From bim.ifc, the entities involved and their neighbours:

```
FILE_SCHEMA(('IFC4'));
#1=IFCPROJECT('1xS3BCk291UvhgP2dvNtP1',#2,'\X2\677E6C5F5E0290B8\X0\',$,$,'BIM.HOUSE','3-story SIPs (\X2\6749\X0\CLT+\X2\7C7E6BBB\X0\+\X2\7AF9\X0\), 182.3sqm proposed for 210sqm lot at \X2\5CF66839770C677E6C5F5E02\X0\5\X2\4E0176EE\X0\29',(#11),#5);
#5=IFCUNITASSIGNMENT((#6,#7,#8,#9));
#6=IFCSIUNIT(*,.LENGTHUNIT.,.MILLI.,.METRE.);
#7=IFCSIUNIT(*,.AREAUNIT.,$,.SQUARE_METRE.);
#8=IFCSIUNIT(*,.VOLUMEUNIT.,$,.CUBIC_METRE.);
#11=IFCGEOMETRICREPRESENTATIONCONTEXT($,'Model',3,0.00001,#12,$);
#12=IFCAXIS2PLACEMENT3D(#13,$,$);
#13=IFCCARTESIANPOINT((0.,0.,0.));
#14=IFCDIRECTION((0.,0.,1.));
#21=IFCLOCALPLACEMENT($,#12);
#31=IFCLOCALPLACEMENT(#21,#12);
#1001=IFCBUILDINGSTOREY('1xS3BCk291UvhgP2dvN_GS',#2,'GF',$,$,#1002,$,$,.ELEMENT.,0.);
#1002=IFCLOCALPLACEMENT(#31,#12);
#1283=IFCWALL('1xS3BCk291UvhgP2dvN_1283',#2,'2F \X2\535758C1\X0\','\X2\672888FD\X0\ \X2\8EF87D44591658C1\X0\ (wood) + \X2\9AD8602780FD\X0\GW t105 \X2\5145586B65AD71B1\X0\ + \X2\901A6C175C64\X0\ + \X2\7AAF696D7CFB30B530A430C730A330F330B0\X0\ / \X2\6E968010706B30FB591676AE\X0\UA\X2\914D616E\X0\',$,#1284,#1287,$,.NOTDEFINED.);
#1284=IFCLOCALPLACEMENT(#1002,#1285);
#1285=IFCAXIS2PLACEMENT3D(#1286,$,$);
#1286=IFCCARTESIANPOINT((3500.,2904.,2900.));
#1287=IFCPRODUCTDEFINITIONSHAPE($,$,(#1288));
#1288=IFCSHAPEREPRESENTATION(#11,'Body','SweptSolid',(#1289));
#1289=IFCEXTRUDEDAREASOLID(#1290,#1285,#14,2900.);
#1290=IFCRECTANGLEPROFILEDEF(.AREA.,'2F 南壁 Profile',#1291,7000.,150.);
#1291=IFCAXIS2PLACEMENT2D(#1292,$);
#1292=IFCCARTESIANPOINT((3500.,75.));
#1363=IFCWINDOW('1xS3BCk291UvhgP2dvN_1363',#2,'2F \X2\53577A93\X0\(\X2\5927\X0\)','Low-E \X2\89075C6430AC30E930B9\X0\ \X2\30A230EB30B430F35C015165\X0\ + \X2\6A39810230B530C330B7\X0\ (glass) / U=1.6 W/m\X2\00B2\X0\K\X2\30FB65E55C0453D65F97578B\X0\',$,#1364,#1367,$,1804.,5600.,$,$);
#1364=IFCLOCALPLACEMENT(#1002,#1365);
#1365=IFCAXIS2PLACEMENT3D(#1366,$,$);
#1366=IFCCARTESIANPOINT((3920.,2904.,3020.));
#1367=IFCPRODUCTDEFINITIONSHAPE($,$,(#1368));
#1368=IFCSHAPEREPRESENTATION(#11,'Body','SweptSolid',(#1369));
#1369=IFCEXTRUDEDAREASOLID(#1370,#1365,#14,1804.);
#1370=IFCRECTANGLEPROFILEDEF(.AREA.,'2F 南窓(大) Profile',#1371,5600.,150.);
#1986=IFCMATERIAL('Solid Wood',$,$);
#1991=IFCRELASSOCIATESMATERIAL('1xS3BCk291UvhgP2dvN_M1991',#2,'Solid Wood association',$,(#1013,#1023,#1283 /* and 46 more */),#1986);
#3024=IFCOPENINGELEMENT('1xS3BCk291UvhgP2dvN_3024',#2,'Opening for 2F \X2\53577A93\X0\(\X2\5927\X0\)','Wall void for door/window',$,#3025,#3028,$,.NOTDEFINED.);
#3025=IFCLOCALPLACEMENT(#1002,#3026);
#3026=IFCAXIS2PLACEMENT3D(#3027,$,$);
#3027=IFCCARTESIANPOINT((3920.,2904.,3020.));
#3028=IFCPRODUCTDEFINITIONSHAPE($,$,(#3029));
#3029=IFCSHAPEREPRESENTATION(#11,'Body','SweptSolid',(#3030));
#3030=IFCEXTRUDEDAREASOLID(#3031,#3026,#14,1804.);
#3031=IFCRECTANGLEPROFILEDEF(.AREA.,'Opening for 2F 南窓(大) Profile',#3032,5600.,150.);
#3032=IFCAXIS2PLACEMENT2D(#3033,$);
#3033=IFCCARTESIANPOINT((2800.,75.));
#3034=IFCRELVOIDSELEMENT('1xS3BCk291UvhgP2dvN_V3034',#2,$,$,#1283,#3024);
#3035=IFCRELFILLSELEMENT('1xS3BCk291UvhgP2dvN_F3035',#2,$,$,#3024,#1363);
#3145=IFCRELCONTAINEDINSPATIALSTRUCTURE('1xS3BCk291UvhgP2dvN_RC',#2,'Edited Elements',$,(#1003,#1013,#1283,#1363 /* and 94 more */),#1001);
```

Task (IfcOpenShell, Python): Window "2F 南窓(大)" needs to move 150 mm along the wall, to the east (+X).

```python
import ifcopenshell
import ifcopenshell.api.geometry
import ifcopenshell.util.placement
import ifcopenshell.util.unit

model = ifcopenshell.open("bim.ifc")
unit_scale = ifcopenshell.util.unit.calculate_unit_scale(model)

window = model.by_guid("1xS3BCk291UvhgP2dvN_1363")
opening = window.FillsVoids[0].RelatingOpeningElement
wall = opening.VoidsElements[0].RelatingBuildingElement

wall_matrix = ifcopenshell.util.placement.get_local_placement(wall.ObjectPlacement)
shift = wall_matrix[:3, 0] * 0.15 / unit_scale
before = ifcopenshell.util.placement.get_local_placement(window.ObjectPlacement)[:3, 3].copy()

# The window is not placed relative to its opening, so move both.
for product in (opening, window):
    matrix = ifcopenshell.util.placement.get_local_placement(product.ObjectPlacement)
    matrix[:3, 3] += shift
    ifcopenshell.api.geometry.edit_object_placement(model, product=product, matrix=matrix, is_si=False)

after = ifcopenshell.util.placement.get_local_placement(window.ObjectPlacement)[:3, 3]
print("window moved by", (after - before).round(3) + 0.0)

model.write("bim_rev.ifc")
```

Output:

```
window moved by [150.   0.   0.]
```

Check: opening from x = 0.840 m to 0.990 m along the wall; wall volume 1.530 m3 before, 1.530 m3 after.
